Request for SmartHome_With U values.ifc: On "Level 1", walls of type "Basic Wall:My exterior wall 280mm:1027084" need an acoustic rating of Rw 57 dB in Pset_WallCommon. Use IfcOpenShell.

First a look at what the model holds.

```python
import ifcopenshell
import ifcopenshell.util.element

model = ifcopenshell.open("SmartHome_With U values.ifc")
print(model.schema)
storey = next(s for s in model.by_type("IfcBuildingStorey") if s.Name == "Level 1")
walls = [e for e in ifcopenshell.util.element.get_decomposition(storey) if e.is_a("IfcWall")]
seen = {}
for e in walls:
    element_type = ifcopenshell.util.element.get_type(e)
    key = (element_type.Name if element_type != e and element_type else None, ifcopenshell.util.element.get_pset(e, "Pset_WallCommon", "AcousticRating"))
    seen[key] = seen.get(key, 0) + 1
for (name, value), count in sorted(seen.items(), key=str):
    print(count, "x", name, "|", value)
```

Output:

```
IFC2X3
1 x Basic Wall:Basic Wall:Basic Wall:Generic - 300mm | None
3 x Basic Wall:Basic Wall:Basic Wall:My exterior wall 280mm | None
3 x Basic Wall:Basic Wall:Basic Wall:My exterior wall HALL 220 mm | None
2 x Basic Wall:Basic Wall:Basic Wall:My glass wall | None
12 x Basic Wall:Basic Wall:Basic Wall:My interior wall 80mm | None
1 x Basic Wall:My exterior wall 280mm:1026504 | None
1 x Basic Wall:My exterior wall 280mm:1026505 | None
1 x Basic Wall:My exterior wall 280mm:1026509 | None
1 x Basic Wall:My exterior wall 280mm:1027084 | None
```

```python
import ifcopenshell
import ifcopenshell.api.pset
import ifcopenshell.util.element

model = ifcopenshell.open("SmartHome_With U values.ifc")

storey = next(s for s in model.by_type("IfcBuildingStorey") if s.Name == "Level 1")
walls = [e for e in ifcopenshell.util.element.get_decomposition(storey) if e.is_a("IfcWall")]

count = 0
for e in walls:
    element_type = ifcopenshell.util.element.get_type(e)
    if element_type in (None, e) or element_type.Name != "Basic Wall:My exterior wall 280mm:1027084":
        continue
    # add_pset returns the element's existing set when there is one.
    pset = ifcopenshell.api.pset.add_pset(model, product=e, name="Pset_WallCommon")
    ifcopenshell.api.pset.edit_pset(model, pset=pset, properties={"AcousticRating": "Rw 57 dB"})
    count += 1

print(count, "walls updated")

model.write("SmartHome_With U values_updated.ifc")
```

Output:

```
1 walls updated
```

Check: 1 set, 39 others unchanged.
